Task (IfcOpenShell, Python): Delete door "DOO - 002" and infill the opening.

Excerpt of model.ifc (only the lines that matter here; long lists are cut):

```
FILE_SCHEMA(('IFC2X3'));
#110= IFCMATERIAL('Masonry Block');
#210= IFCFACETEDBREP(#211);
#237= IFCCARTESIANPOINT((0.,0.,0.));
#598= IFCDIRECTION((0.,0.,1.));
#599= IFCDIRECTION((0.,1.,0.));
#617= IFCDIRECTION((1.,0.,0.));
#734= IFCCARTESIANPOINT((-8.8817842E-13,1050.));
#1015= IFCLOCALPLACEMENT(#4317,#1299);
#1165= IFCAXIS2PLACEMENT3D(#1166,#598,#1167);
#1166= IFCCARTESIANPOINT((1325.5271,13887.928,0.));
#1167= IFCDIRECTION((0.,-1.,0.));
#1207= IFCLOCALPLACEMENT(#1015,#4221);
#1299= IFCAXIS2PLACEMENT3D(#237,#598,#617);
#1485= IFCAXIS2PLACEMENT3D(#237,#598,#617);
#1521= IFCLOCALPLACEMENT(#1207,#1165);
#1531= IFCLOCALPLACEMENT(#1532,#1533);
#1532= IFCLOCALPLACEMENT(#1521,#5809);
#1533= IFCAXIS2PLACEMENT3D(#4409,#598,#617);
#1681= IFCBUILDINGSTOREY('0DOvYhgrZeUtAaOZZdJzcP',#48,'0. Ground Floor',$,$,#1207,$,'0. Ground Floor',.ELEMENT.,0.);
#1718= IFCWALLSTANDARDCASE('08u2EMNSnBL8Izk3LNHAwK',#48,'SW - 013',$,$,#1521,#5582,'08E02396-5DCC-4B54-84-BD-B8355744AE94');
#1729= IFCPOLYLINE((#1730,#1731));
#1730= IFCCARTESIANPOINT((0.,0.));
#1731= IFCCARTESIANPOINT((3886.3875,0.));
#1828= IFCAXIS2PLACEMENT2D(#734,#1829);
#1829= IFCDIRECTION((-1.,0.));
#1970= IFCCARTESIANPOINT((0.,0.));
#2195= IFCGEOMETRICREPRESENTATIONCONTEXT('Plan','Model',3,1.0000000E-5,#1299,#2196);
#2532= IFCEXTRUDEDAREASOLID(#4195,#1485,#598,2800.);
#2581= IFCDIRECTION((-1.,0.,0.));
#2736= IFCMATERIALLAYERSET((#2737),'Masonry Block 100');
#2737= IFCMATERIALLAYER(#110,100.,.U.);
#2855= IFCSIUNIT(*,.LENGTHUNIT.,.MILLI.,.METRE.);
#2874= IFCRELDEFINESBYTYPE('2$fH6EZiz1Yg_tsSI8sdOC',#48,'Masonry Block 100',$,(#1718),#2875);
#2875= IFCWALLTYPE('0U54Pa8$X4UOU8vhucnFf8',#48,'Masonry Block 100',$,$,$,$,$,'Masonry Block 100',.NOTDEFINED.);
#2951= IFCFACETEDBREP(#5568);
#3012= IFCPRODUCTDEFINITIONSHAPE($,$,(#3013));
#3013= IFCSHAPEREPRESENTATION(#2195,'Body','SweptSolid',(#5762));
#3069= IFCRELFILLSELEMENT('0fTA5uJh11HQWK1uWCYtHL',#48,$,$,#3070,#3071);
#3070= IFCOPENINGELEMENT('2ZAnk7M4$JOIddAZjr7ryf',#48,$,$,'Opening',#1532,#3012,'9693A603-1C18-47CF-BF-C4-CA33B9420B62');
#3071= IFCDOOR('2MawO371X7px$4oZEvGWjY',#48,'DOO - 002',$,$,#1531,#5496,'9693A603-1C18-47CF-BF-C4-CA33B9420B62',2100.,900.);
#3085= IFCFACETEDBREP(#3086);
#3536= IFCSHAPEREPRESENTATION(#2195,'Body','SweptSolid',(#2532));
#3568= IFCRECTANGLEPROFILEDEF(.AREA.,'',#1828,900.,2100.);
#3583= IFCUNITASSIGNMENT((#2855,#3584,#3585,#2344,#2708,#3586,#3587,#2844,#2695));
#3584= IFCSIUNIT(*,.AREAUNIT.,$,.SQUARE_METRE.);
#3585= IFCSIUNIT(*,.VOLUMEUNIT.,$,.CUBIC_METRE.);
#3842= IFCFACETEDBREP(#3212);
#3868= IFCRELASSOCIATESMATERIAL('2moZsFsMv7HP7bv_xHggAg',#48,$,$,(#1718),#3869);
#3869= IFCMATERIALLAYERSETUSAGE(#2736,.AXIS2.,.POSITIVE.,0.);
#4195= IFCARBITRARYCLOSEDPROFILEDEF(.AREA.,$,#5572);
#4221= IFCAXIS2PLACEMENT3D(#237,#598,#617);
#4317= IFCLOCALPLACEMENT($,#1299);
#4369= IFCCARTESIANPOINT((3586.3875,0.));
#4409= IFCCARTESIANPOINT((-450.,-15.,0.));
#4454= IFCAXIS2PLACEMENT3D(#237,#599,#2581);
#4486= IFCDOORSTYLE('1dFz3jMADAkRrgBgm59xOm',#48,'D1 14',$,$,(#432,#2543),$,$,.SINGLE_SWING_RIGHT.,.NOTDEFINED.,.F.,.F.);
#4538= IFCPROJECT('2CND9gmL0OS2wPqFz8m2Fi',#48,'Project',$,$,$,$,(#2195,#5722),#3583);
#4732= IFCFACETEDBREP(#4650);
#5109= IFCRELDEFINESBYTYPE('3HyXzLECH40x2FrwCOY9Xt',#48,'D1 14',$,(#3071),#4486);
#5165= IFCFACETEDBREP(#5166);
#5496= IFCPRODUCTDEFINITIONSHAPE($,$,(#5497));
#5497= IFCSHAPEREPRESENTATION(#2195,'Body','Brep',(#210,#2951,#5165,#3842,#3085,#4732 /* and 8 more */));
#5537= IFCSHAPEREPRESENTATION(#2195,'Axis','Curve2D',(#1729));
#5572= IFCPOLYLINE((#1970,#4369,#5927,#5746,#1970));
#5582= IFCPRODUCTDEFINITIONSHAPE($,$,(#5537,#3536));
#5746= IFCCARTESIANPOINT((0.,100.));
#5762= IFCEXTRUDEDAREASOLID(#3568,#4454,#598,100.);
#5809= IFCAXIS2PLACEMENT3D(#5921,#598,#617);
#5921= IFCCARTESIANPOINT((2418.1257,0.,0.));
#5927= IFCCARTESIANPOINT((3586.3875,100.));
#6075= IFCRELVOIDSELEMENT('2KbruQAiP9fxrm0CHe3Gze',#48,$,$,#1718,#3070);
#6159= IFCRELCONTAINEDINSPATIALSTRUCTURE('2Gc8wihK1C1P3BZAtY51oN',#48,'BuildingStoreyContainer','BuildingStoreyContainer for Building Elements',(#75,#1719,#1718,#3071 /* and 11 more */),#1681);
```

```python
import ifcopenshell
import ifcopenshell.api.feature
import ifcopenshell.api.root
import ifcopenshell.geom
import ifcopenshell.util.shape

model = ifcopenshell.open("model.ifc")
settings = ifcopenshell.geom.settings()


def volume(element):
    """Net volume in cubic metres, openings subtracted."""
    shape = ifcopenshell.geom.create_shape(settings, element)
    return ifcopenshell.util.shape.get_volume(shape.geometry)


door = model.by_id(3071)
opening = door.FillsVoids[0].RelatingOpeningElement
wall = opening.VoidsElements[0].RelatingBuildingElement
before = volume(wall)

ifcopenshell.api.root.remove_product(model, product=door)
ifcopenshell.api.feature.remove_feature(model, feature=opening)

after = volume(wall)

print(f"wall volume {before:.3f} -> {after:.3f} m3")

model.write("model_v2.ifc")
```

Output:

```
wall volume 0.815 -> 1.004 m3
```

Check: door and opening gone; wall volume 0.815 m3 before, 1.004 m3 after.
